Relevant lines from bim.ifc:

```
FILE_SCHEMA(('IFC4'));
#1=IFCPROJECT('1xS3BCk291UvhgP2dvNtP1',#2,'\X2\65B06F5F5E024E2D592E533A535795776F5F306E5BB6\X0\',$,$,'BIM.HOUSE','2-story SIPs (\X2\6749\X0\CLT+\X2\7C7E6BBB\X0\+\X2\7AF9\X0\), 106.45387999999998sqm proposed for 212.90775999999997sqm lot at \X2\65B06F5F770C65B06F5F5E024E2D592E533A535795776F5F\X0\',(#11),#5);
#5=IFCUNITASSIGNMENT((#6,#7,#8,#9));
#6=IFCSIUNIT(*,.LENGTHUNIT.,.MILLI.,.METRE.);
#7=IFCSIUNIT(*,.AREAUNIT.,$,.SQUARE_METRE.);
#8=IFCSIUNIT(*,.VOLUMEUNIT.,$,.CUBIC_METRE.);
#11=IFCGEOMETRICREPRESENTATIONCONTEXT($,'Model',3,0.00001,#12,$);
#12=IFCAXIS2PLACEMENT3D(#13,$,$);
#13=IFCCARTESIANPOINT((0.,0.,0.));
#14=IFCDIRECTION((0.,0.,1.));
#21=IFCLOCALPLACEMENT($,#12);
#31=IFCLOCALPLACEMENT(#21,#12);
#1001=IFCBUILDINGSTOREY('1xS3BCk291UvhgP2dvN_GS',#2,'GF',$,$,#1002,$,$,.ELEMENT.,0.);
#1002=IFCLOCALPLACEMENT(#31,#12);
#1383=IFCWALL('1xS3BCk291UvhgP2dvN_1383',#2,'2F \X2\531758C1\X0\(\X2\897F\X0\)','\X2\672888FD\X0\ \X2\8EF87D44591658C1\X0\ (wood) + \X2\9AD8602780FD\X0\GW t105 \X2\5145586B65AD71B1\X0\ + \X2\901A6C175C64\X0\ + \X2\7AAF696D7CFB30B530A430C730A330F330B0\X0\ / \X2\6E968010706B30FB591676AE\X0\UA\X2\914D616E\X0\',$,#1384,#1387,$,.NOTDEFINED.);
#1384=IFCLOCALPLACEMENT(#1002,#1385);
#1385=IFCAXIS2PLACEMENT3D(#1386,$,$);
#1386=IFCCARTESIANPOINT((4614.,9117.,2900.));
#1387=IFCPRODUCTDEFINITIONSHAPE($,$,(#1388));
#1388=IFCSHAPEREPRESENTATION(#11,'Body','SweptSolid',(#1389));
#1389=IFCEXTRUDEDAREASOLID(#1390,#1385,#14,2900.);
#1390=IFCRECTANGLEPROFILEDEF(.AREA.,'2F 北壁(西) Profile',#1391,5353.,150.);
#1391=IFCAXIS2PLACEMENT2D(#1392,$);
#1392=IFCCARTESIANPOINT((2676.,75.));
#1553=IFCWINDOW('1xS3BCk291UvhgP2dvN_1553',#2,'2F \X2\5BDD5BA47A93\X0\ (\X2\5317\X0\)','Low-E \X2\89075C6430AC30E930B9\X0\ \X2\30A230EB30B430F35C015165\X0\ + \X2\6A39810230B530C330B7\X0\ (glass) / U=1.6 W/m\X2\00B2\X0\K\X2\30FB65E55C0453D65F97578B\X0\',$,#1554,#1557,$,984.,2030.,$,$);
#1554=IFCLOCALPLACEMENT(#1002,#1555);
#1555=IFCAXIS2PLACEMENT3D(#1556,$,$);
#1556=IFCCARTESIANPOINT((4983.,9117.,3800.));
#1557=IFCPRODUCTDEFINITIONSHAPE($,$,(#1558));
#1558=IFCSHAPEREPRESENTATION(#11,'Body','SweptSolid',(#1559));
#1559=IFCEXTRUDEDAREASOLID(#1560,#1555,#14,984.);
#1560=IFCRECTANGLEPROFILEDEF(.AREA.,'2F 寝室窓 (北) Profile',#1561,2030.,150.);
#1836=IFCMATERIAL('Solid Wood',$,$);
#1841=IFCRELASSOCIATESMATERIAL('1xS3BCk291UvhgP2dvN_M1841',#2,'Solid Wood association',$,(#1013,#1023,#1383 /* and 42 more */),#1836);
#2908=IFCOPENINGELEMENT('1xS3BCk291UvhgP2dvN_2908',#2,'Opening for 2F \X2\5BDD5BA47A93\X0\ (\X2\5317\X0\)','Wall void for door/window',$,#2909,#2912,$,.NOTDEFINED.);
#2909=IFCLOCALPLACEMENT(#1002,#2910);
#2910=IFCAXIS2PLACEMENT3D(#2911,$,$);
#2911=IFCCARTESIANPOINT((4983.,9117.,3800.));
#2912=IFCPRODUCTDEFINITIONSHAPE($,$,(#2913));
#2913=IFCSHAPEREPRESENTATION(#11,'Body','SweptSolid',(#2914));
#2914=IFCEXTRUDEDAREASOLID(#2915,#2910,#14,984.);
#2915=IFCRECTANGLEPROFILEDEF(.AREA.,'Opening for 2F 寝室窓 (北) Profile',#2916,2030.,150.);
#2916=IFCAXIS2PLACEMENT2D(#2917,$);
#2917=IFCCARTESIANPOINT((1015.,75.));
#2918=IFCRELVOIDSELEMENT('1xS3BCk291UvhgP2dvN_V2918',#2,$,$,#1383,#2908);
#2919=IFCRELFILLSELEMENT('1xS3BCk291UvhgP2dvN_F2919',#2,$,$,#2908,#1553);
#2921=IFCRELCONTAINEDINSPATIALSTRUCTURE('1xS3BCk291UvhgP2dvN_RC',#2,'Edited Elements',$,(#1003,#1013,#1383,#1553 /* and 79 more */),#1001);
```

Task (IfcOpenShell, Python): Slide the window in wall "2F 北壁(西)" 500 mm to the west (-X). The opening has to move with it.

```python
import ifcopenshell
import ifcopenshell.api.geometry
import ifcopenshell.util.placement

model = ifcopenshell.open("bim.ifc")

window = model.by_guid("1xS3BCk291UvhgP2dvN_1553")
opening = window.FillsVoids[0].RelatingOpeningElement
wall = opening.VoidsElements[0].RelatingBuildingElement

wall_matrix = ifcopenshell.util.placement.get_local_placement(wall.ObjectPlacement)
shift = wall_matrix[:3, 0] * -500.0
before = ifcopenshell.util.placement.get_local_placement(window.ObjectPlacement)[:3, 3].copy()

# The window is not placed relative to its opening, so move both.
for product in (opening, window):
    matrix = ifcopenshell.util.placement.get_local_placement(product.ObjectPlacement)
    matrix[:3, 3] += shift
    ifcopenshell.api.geometry.edit_object_placement(model, product=product, matrix=matrix, is_si=False)

after = ifcopenshell.util.placement.get_local_placement(window.ObjectPlacement)[:3, 3]
print("window moved by", (after - before).round(3) + 0.0)

model.write("bim-out.ifc")
```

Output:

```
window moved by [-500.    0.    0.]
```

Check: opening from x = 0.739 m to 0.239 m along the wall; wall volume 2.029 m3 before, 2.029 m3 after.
